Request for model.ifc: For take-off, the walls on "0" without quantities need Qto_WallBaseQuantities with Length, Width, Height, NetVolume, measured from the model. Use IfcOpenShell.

First a look at what the model holds.

```python
import ifcopenshell
import ifcopenshell.util.element
import ifcopenshell.util.unit

model = ifcopenshell.open("model.ifc")
print(model.schema)
for unit_type in ("LENGTHUNIT", "AREAUNIT", "VOLUMEUNIT"):
    print(unit_type, ifcopenshell.util.unit.calculate_unit_scale(model, unit_type))
storey = next(s for s in model.by_type("IfcBuildingStorey") if s.Name == "0")
walls = [e for e in ifcopenshell.util.element.get_decomposition(storey) if e.is_a("IfcWall")]
for e in sorted(walls, key=lambda e: e.id()):
    print(e.id(), e.is_a(), e.Name, list(ifcopenshell.util.element.get_psets(e, qtos_only=True)), sep=" | ")
```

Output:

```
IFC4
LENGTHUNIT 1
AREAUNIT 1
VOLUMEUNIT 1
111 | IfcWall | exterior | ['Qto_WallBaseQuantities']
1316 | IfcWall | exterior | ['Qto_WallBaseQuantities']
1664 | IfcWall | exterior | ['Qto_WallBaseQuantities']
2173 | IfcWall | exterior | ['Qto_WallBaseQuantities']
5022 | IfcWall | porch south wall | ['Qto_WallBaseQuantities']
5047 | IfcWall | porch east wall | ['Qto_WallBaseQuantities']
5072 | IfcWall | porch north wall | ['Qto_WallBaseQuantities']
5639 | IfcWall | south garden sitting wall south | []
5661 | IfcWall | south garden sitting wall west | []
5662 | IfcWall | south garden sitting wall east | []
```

```python
import ifcopenshell
import ifcopenshell.api.pset
import ifcopenshell.geom
import ifcopenshell.util.element
import ifcopenshell.util.shape
import ifcopenshell.util.unit

model = ifcopenshell.open("model.ifc")
unit_scale = ifcopenshell.util.unit.calculate_unit_scale(model)
volume_scale = ifcopenshell.util.unit.calculate_unit_scale(model, "VOLUMEUNIT")
settings = ifcopenshell.geom.settings()

storey = next(s for s in model.by_type("IfcBuildingStorey") if s.Name == "0")
walls = [e for e in ifcopenshell.util.element.get_decomposition(storey) if e.is_a("IfcWall")]

for e in sorted(walls, key=lambda e: e.id()):
    if ifcopenshell.util.element.get_psets(e, qtos_only=True, should_inherit=False):
        continue
    # Geometry comes back in metres, in the element's own axes.
    shape = ifcopenshell.geom.create_shape(settings, e)
    values = {
        "Length": ifcopenshell.util.shape.get_x(shape.geometry) / unit_scale,
        "Width": ifcopenshell.util.shape.get_y(shape.geometry) / unit_scale,
        "Height": ifcopenshell.util.shape.get_z(shape.geometry) / unit_scale,
        "NetVolume": ifcopenshell.util.shape.get_volume(shape.geometry) / volume_scale,
    }
    qto = ifcopenshell.api.pset.add_qto(model, product=e, name="Qto_WallBaseQuantities")
    ifcopenshell.api.pset.edit_qto(model, qto=qto, properties=values)
    print(e.id(), {k: round(v, 3) for k, v in values.items()})

model.write("model_rev.ifc")
```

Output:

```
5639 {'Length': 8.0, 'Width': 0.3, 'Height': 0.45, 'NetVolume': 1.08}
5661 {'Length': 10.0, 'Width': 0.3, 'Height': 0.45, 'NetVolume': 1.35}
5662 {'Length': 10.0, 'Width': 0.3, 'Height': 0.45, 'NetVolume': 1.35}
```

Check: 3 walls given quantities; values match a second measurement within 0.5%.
